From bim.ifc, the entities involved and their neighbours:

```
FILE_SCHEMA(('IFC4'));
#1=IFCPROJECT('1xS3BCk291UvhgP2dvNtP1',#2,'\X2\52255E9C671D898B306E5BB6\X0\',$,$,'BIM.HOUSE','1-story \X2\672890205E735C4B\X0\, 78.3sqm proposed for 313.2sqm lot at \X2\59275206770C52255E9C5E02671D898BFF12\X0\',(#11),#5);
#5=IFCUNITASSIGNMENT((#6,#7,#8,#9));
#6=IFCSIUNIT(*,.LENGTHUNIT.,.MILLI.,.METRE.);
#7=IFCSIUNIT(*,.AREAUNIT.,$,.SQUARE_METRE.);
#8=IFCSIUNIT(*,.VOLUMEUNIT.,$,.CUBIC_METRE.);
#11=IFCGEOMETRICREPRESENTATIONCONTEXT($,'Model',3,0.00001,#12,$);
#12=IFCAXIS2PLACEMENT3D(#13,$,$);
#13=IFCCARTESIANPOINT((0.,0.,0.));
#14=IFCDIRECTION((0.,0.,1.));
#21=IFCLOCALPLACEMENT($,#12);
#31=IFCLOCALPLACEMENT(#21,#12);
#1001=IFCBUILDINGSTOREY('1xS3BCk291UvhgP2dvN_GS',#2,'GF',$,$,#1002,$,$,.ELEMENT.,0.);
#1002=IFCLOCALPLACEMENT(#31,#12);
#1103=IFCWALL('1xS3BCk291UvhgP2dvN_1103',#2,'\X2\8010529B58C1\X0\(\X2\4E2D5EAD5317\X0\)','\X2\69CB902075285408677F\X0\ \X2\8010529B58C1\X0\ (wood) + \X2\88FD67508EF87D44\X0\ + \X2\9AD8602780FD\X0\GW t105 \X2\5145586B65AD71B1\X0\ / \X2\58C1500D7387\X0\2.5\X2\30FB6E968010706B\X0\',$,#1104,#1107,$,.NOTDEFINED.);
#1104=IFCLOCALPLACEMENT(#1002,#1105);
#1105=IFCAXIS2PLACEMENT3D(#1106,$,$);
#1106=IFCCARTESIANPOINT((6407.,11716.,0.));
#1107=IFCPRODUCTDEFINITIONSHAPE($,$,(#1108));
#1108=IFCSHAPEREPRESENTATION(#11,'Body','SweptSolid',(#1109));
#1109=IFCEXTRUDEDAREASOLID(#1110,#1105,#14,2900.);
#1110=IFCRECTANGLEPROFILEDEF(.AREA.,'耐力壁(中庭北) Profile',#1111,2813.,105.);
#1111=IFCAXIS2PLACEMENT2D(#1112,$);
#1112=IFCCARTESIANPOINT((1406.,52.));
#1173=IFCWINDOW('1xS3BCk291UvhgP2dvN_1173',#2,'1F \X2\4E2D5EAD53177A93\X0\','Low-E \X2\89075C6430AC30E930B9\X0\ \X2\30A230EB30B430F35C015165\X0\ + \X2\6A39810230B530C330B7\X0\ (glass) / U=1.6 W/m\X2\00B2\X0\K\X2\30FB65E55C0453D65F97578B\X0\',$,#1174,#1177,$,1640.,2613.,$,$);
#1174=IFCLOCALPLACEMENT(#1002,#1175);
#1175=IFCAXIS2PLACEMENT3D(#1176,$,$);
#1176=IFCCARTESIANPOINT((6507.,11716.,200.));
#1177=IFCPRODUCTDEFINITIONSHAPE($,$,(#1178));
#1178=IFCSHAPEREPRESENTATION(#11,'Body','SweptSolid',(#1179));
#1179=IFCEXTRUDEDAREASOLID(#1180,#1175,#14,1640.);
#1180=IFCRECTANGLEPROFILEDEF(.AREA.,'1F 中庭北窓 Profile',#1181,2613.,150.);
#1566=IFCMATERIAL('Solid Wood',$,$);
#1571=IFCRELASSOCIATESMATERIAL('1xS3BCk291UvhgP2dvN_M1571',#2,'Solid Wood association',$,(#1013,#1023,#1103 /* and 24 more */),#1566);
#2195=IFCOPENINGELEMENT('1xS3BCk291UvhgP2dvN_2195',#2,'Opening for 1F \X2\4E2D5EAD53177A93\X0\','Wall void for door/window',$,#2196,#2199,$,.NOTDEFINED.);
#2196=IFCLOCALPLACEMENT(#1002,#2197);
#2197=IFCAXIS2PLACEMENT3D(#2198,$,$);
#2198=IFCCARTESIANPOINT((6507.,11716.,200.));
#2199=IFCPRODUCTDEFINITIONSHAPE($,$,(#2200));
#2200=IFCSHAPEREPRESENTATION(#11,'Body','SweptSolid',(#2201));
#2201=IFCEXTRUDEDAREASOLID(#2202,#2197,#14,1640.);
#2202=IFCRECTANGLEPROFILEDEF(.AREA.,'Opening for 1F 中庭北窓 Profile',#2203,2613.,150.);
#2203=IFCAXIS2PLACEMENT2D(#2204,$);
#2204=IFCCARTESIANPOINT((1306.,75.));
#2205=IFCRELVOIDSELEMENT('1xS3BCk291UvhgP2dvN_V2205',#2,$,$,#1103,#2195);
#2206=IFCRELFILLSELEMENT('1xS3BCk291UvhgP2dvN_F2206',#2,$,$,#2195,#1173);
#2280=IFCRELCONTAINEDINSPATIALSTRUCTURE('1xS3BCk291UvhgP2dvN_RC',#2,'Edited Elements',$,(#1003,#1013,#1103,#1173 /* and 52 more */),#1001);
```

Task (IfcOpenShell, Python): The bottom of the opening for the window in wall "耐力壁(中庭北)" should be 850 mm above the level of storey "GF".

```python
import numpy as np
import ifcopenshell
import ifcopenshell.api.geometry
import ifcopenshell.geom
import ifcopenshell.util.element
import ifcopenshell.util.placement
import ifcopenshell.util.shape
import ifcopenshell.util.unit

model = ifcopenshell.open("bim.ifc")
unit_scale = ifcopenshell.util.unit.calculate_unit_scale(model)

window = model.by_guid("1xS3BCk291UvhgP2dvN_1173")
opening = window.FillsVoids[0].RelatingOpeningElement
storey = ifcopenshell.util.element.get_container(window, ifc_class="IfcBuildingStorey")
level = ifcopenshell.util.placement.get_local_placement(storey.ObjectPlacement)[2, 3]

# The opening's origin need not be at the sill, so measure its lowest point.
shape = ifcopenshell.geom.create_shape(ifcopenshell.geom.settings(), opening)
bottom = ifcopenshell.util.shape.get_shape_bottom_elevation(shape, shape.geometry) / unit_scale
dz = level + 0.85 / unit_scale - bottom

shift = np.array([0.0, 0.0, dz])
# The window is not placed relative to its opening, so move both.
for product in (opening, window):
    matrix = ifcopenshell.util.placement.get_local_placement(product.ObjectPlacement)
    matrix[:3, 3] += shift
    ifcopenshell.api.geometry.edit_object_placement(model, product=product, matrix=matrix, is_si=False)

print(f"moved by {dz * unit_scale:+.3f} m")

model.write("bim_rev.ifc")
```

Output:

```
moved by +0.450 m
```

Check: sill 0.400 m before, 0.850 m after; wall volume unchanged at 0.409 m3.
